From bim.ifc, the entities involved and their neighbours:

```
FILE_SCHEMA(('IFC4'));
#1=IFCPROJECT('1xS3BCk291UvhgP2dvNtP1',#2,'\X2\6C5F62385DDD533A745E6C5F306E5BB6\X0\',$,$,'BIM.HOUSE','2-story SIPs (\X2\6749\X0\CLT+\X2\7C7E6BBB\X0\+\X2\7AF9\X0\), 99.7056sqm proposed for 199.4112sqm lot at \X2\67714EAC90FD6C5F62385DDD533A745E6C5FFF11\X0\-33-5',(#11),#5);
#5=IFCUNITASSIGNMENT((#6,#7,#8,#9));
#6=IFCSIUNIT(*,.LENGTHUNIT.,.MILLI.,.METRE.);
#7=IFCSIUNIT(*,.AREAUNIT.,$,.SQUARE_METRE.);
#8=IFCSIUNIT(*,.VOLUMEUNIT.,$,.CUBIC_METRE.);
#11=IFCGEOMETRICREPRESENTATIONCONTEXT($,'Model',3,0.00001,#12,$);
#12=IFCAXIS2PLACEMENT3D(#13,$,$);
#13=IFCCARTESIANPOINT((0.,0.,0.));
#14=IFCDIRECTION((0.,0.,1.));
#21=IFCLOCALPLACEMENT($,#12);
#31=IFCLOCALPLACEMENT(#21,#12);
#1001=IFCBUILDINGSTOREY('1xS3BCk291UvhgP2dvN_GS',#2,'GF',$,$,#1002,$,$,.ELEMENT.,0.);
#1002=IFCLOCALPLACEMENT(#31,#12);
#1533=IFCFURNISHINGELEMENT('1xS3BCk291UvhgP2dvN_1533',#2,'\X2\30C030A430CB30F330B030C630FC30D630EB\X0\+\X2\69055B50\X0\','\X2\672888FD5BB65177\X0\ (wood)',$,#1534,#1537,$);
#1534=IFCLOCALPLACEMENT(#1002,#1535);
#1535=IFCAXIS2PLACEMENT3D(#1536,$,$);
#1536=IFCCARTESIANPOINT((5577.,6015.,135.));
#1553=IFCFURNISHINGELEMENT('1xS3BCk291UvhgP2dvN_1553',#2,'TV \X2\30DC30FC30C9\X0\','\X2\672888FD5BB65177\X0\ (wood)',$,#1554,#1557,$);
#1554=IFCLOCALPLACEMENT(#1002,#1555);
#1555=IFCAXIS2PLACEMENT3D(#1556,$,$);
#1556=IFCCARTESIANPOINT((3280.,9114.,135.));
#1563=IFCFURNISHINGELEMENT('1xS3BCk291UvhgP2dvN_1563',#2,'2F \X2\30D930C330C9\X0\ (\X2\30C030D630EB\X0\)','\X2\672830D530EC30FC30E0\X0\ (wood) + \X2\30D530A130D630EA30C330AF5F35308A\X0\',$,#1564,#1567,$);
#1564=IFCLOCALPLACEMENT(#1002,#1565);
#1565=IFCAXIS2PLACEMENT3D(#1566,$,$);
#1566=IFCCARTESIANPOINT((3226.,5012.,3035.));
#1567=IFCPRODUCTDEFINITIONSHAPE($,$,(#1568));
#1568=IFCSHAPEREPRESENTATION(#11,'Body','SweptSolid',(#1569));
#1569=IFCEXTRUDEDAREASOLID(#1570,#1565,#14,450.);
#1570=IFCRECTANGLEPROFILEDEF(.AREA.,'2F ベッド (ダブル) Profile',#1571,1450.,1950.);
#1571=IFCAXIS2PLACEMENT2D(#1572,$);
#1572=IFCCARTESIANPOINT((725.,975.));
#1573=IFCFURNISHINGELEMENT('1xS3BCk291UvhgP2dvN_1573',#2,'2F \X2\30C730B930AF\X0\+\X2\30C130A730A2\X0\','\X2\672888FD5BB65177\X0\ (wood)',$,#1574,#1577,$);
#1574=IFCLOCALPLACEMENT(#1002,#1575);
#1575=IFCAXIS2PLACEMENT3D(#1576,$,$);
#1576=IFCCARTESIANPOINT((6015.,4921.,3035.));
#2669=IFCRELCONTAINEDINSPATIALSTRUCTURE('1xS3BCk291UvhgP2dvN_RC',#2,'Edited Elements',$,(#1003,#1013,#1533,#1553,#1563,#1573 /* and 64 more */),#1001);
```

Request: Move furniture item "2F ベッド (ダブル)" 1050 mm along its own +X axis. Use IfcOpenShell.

```python
import ifcopenshell
import ifcopenshell.api.geometry
import ifcopenshell.util.placement
import ifcopenshell.util.unit

model = ifcopenshell.open("bim.ifc")
unit_scale = ifcopenshell.util.unit.calculate_unit_scale(model)

item = model.by_guid("1xS3BCk291UvhgP2dvN_1563")
matrix = ifcopenshell.util.placement.get_local_placement(item.ObjectPlacement)
matrix[:3, 3] += matrix[:3, 0] * 1.05 / unit_scale
ifcopenshell.api.geometry.edit_object_placement(model, product=item, matrix=matrix, is_si=False)

print(ifcopenshell.util.placement.get_local_placement(item.ObjectPlacement).round(3) + 0.0)

model.write("bim_rev.ifc")
```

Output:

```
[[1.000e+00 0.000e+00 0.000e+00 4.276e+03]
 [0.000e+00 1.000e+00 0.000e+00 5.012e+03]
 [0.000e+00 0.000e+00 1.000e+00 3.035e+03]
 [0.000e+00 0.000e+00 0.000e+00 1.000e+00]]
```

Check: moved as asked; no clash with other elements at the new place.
